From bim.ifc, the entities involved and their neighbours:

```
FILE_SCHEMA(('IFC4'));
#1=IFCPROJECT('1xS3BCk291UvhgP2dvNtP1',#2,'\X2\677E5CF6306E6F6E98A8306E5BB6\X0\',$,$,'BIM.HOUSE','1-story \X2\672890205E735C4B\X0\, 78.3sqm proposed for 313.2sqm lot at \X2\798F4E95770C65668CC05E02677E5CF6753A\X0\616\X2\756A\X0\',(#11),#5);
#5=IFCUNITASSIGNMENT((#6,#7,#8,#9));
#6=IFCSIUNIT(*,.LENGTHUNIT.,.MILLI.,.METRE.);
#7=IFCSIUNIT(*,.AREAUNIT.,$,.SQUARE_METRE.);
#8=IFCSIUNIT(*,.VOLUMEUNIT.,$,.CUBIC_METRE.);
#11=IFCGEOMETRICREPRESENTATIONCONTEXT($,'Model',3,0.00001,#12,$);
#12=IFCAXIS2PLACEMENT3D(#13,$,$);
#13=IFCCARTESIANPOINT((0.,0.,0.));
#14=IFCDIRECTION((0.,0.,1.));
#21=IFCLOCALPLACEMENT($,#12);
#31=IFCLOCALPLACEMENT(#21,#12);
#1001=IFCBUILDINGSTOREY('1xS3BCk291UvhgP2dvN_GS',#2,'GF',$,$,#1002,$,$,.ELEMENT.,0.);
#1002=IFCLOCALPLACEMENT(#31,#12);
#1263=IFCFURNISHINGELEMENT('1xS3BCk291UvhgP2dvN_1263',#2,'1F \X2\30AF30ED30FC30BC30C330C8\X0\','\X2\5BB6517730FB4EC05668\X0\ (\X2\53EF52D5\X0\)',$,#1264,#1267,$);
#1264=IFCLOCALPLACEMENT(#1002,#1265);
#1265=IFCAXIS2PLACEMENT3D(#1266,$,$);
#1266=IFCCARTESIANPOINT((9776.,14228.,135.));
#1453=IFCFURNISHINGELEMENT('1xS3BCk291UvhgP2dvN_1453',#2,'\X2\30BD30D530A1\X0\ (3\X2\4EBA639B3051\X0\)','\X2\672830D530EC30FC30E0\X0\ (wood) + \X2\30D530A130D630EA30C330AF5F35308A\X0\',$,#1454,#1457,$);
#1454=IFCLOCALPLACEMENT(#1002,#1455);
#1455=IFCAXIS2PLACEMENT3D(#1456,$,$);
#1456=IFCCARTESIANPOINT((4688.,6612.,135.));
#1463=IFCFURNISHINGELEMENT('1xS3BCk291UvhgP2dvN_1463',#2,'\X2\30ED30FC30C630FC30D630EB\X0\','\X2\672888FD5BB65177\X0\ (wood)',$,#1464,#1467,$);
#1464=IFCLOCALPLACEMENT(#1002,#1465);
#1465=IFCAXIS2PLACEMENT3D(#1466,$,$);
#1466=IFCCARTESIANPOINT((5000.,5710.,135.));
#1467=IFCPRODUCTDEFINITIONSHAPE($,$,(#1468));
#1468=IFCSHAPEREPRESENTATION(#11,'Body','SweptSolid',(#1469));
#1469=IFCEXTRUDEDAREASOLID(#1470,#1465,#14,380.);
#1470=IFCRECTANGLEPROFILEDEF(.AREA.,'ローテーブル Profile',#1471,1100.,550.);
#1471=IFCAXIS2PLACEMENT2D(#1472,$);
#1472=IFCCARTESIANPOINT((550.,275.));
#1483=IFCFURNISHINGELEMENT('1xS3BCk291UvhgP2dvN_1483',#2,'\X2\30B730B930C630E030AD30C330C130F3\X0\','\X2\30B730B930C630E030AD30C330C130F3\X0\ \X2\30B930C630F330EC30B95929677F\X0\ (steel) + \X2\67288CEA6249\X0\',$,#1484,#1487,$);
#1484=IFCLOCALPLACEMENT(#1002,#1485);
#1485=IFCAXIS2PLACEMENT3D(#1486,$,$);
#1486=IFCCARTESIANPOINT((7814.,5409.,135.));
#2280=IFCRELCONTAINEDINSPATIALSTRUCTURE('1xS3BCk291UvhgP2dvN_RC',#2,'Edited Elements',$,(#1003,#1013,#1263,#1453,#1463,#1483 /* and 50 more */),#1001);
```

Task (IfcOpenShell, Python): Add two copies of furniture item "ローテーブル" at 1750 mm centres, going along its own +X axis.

```python
import ifcopenshell
import ifcopenshell.api.geometry
import ifcopenshell.api.root
import ifcopenshell.util.element
import ifcopenshell.util.placement
import ifcopenshell.util.unit

model = ifcopenshell.open("bim.ifc")
unit_scale = ifcopenshell.util.unit.calculate_unit_scale(model)


def reuse_history(source, copy):
    """copy_class also copies each property set's owner history, people and application; keep the originals."""
    for rel in copy.IsDefinedBy:
        if rel.is_a("IfcRelDefinesByProperties") and (history := rel.RelatingPropertyDefinition.OwnerHistory):
            rel.RelatingPropertyDefinition.OwnerHistory = source.OwnerHistory
            ifcopenshell.util.element.remove_deep2(model, history)


source = model.by_guid("1xS3BCk291UvhgP2dvN_1463")
base = ifcopenshell.util.placement.get_local_placement(source.ObjectPlacement)
step = base[:3, 0] * 1.75 / unit_scale

for i in range(1, 3):
    copy = ifcopenshell.api.root.copy_class(model, product=source)
    copy.Representation = ifcopenshell.util.element.copy_deep(
        model, source.Representation, exclude=["IfcGeometricRepresentationContext", "IfcRepresentationMap"]
    )
    reuse_history(source, copy)
    matrix = base.copy()
    matrix[:3, 3] += i * step
    print("added at", matrix[:3, 3].round(3) + 0.0)
    ifcopenshell.api.geometry.edit_object_placement(model, product=copy, matrix=matrix, is_si=False)

model.write("bim_updated.ifc")
```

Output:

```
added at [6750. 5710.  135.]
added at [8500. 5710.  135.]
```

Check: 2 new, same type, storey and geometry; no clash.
